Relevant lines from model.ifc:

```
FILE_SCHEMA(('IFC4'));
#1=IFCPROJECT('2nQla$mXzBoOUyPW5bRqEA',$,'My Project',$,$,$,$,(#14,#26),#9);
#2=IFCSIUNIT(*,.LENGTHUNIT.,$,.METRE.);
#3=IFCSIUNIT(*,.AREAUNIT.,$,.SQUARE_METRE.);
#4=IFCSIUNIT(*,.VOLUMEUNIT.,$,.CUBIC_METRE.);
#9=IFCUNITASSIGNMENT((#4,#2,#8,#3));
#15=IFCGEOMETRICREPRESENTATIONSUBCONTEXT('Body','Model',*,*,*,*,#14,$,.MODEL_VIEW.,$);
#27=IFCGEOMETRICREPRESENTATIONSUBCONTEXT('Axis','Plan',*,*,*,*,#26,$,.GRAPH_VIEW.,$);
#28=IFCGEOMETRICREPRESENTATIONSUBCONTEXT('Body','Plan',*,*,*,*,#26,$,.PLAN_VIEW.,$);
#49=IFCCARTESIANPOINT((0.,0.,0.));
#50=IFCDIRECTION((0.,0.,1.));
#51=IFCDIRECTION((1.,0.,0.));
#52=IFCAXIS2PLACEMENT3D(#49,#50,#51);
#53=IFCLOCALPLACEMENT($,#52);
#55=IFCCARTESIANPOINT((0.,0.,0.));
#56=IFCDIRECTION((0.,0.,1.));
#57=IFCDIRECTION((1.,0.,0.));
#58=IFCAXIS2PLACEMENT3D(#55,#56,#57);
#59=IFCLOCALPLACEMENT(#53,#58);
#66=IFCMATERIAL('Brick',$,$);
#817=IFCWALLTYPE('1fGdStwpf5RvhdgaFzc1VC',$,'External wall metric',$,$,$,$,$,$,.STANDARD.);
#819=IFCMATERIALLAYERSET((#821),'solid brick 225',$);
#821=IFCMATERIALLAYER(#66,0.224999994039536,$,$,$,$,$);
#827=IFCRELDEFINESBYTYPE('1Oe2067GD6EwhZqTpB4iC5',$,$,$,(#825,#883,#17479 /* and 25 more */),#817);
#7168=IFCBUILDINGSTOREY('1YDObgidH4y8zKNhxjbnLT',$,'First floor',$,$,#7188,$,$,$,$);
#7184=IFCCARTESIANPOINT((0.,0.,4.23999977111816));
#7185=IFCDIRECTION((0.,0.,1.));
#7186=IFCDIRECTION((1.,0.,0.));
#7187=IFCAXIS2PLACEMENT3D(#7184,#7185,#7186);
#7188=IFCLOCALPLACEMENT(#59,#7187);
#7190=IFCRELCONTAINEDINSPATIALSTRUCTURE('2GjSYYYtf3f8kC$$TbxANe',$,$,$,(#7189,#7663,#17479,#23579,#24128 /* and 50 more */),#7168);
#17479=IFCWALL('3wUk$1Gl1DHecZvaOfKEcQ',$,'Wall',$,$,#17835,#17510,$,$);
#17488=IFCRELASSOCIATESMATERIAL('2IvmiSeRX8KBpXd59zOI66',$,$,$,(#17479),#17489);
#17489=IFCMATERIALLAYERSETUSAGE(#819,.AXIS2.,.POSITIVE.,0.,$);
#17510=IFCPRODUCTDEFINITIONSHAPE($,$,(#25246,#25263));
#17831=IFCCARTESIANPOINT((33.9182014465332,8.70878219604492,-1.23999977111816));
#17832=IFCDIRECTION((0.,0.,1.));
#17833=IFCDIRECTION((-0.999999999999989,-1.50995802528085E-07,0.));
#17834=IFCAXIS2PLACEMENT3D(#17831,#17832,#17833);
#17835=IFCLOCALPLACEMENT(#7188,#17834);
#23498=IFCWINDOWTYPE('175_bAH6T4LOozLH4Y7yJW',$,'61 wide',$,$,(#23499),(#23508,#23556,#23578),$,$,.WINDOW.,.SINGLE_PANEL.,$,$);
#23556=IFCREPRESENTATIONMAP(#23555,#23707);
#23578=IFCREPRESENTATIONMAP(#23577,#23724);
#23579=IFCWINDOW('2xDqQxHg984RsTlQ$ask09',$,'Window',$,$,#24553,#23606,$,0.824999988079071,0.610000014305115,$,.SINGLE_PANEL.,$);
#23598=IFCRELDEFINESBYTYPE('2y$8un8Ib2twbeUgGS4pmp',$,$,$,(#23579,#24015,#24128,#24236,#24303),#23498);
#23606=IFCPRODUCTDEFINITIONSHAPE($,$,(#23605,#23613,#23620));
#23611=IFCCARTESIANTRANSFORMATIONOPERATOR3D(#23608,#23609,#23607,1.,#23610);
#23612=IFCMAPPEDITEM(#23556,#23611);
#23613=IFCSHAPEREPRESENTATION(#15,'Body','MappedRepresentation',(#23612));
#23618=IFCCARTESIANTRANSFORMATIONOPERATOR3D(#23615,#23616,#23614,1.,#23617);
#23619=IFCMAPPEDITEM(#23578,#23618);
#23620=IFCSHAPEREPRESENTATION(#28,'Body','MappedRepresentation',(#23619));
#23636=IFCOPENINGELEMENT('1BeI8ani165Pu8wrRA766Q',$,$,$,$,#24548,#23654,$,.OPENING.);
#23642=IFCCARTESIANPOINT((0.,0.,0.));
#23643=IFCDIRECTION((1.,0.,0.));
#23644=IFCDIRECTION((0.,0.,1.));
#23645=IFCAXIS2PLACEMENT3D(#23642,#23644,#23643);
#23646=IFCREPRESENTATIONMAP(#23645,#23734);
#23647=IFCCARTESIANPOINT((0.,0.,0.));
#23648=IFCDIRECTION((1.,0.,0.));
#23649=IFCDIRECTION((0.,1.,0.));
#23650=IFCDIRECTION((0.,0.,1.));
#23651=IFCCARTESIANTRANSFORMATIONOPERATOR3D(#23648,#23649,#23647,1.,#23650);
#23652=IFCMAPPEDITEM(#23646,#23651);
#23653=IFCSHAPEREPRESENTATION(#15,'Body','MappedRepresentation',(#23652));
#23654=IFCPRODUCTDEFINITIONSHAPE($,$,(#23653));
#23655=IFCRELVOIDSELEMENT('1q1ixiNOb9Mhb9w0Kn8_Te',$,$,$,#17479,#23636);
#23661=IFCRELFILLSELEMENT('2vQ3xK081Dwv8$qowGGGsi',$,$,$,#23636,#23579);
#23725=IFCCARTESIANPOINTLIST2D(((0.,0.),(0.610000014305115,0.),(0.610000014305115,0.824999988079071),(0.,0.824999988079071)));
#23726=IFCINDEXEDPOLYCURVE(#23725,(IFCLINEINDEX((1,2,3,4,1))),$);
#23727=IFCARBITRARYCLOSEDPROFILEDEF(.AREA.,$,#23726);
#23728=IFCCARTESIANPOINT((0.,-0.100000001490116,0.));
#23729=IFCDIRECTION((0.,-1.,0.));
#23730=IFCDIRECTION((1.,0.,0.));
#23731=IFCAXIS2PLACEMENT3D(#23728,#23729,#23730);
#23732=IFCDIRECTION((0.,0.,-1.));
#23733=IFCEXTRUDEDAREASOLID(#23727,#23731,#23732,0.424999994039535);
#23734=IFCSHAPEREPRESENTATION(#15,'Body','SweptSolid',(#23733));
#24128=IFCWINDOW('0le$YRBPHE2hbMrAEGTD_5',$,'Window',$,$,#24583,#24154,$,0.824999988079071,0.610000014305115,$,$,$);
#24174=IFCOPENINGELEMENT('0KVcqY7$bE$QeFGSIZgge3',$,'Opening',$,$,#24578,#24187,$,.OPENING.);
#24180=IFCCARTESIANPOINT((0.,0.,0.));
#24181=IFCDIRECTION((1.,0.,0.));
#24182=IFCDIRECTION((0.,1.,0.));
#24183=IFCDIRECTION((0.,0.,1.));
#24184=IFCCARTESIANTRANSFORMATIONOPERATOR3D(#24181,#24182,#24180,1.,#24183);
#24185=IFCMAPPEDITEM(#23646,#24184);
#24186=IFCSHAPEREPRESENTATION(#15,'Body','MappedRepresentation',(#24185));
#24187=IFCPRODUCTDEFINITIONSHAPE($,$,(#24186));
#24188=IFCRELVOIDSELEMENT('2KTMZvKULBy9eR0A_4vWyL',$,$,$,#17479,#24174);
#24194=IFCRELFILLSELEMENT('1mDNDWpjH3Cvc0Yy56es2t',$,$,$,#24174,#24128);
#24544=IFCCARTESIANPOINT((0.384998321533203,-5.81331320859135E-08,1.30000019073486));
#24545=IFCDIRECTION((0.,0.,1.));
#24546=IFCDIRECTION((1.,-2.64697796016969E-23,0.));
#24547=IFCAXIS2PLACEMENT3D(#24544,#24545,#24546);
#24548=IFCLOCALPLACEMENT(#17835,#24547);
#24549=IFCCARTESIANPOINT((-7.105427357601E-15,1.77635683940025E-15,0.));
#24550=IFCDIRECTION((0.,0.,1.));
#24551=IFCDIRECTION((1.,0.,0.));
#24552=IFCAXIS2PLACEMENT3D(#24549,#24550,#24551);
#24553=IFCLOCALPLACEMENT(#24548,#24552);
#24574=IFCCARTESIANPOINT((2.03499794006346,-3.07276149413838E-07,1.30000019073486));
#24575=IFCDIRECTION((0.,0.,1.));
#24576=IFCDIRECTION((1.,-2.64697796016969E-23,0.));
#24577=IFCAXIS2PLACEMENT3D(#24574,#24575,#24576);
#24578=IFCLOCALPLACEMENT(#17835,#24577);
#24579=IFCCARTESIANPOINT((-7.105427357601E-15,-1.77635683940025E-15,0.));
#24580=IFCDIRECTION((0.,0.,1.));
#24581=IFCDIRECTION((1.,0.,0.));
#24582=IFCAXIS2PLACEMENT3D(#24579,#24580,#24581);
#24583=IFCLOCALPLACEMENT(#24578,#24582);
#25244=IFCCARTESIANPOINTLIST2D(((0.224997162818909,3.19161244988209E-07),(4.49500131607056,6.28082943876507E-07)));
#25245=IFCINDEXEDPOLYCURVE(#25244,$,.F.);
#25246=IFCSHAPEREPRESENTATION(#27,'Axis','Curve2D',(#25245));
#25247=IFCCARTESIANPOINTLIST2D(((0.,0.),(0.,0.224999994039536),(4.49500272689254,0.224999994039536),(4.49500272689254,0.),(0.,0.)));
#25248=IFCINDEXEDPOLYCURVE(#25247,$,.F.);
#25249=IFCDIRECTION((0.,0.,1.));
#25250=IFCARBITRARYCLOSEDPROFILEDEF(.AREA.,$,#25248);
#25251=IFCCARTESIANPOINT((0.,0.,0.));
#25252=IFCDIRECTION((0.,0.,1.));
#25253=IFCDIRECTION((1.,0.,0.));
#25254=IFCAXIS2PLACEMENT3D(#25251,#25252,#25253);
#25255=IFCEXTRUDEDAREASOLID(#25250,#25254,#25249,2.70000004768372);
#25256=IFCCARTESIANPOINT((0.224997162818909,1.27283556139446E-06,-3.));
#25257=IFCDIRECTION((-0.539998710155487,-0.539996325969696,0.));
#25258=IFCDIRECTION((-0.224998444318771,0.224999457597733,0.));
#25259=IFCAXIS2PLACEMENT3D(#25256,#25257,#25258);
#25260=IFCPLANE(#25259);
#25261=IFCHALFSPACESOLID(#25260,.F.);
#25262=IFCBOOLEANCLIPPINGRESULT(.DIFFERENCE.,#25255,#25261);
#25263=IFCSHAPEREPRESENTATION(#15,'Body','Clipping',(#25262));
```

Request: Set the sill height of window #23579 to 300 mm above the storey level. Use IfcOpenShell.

```python
import numpy as np
import ifcopenshell
import ifcopenshell.api.geometry
import ifcopenshell.geom
import ifcopenshell.util.element
import ifcopenshell.util.placement
import ifcopenshell.util.shape
import ifcopenshell.util.unit

model = ifcopenshell.open("model.ifc")
unit_scale = ifcopenshell.util.unit.calculate_unit_scale(model)

window = model.by_id(23579)
opening = window.FillsVoids[0].RelatingOpeningElement
storey = ifcopenshell.util.element.get_container(window, ifc_class="IfcBuildingStorey")
level = ifcopenshell.util.placement.get_local_placement(storey.ObjectPlacement)[2, 3]

# The opening's origin need not be at the sill, so measure its lowest point.
shape = ifcopenshell.geom.create_shape(ifcopenshell.geom.settings(), opening)
bottom = ifcopenshell.util.shape.get_shape_bottom_elevation(shape, shape.geometry) / unit_scale
dz = level + 0.3 / unit_scale - bottom

shift = np.array([0.0, 0.0, dz])
# The window is placed relative to its opening, so it follows when the opening moves.
matrix = ifcopenshell.util.placement.get_local_placement(opening.ObjectPlacement)
matrix[:3, 3] += shift
ifcopenshell.api.geometry.edit_object_placement(
    model, product=opening, matrix=matrix, is_si=False, should_transform_children=True
)

print(f"moved by {dz * unit_scale:+.3f} m")

model.write("model_v2.ifc")
```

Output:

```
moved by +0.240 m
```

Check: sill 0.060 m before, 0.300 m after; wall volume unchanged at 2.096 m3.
